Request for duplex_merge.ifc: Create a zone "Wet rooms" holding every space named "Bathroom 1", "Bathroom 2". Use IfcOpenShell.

First a look at what the model holds.

```python
import ifcopenshell

model = ifcopenshell.open("duplex_merge.ifc")
print(model.schema)
seen = {}
for space in model.by_type("IfcSpace"):
    seen[space.LongName] = seen.get(space.LongName, 0) + 1
for name, count in sorted(seen.items(), key=str):
    print(count, "x", name)
print("zones:", [z.Name for z in model.by_type("IfcZone")][:20])
```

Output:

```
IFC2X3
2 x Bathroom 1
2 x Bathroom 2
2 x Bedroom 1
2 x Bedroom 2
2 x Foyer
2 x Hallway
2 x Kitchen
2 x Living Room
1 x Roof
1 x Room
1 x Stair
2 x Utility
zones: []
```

```python
import ifcopenshell
import ifcopenshell.api.group
import ifcopenshell.api.root

model = ifcopenshell.open("duplex_merge.ifc")

names = {"Bathroom 1", "Bathroom 2"}
spaces = [s for s in model.by_type("IfcSpace") if s.LongName in names]

zone = ifcopenshell.api.root.create_entity(model, ifc_class="IfcZone", name="Wet rooms")
ifcopenshell.api.group.assign_group(model, products=spaces, group=zone)
print(len(spaces), "spaces in", zone.Name)

model.write("duplex_merge_v2.ifc")
```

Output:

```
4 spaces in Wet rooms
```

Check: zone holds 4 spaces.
